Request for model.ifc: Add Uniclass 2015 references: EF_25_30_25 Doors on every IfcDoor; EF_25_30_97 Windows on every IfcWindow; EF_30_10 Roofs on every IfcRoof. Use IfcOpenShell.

First a look at what the model holds.

```python
import ifcopenshell

model = ifcopenshell.open("model.ifc")
print(model.schema)
print("classifications:", [c.Name for c in model.by_type("IfcClassification")])
for ifc_class in ("IfcDoor", "IfcRoof", "IfcStair", "IfcWall", "IfcWindow"):
    print(ifc_class, len(model.by_type(ifc_class)))
```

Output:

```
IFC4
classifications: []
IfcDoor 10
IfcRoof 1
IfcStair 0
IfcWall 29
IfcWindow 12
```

```python
import ifcopenshell
import ifcopenshell.api.classification

model = ifcopenshell.open("model.ifc")

system = ifcopenshell.api.classification.add_classification(model, classification="Uniclass 2015")

codes = {
    "IfcDoor": ("EF_25_30_25", "Doors"),
    "IfcWindow": ("EF_25_30_97", "Windows"),
    "IfcRoof": ("EF_30_10", "Roofs"),
}
for ifc_class, (code, name) in codes.items():
    products = model.by_type(ifc_class)
    ifcopenshell.api.classification.add_reference(
        model, products=products, classification=system, identification=code, name=name
    )
    print(code, len(products))

model.write("model_edited.ifc")
```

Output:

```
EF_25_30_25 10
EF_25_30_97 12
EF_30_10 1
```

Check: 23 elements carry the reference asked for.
